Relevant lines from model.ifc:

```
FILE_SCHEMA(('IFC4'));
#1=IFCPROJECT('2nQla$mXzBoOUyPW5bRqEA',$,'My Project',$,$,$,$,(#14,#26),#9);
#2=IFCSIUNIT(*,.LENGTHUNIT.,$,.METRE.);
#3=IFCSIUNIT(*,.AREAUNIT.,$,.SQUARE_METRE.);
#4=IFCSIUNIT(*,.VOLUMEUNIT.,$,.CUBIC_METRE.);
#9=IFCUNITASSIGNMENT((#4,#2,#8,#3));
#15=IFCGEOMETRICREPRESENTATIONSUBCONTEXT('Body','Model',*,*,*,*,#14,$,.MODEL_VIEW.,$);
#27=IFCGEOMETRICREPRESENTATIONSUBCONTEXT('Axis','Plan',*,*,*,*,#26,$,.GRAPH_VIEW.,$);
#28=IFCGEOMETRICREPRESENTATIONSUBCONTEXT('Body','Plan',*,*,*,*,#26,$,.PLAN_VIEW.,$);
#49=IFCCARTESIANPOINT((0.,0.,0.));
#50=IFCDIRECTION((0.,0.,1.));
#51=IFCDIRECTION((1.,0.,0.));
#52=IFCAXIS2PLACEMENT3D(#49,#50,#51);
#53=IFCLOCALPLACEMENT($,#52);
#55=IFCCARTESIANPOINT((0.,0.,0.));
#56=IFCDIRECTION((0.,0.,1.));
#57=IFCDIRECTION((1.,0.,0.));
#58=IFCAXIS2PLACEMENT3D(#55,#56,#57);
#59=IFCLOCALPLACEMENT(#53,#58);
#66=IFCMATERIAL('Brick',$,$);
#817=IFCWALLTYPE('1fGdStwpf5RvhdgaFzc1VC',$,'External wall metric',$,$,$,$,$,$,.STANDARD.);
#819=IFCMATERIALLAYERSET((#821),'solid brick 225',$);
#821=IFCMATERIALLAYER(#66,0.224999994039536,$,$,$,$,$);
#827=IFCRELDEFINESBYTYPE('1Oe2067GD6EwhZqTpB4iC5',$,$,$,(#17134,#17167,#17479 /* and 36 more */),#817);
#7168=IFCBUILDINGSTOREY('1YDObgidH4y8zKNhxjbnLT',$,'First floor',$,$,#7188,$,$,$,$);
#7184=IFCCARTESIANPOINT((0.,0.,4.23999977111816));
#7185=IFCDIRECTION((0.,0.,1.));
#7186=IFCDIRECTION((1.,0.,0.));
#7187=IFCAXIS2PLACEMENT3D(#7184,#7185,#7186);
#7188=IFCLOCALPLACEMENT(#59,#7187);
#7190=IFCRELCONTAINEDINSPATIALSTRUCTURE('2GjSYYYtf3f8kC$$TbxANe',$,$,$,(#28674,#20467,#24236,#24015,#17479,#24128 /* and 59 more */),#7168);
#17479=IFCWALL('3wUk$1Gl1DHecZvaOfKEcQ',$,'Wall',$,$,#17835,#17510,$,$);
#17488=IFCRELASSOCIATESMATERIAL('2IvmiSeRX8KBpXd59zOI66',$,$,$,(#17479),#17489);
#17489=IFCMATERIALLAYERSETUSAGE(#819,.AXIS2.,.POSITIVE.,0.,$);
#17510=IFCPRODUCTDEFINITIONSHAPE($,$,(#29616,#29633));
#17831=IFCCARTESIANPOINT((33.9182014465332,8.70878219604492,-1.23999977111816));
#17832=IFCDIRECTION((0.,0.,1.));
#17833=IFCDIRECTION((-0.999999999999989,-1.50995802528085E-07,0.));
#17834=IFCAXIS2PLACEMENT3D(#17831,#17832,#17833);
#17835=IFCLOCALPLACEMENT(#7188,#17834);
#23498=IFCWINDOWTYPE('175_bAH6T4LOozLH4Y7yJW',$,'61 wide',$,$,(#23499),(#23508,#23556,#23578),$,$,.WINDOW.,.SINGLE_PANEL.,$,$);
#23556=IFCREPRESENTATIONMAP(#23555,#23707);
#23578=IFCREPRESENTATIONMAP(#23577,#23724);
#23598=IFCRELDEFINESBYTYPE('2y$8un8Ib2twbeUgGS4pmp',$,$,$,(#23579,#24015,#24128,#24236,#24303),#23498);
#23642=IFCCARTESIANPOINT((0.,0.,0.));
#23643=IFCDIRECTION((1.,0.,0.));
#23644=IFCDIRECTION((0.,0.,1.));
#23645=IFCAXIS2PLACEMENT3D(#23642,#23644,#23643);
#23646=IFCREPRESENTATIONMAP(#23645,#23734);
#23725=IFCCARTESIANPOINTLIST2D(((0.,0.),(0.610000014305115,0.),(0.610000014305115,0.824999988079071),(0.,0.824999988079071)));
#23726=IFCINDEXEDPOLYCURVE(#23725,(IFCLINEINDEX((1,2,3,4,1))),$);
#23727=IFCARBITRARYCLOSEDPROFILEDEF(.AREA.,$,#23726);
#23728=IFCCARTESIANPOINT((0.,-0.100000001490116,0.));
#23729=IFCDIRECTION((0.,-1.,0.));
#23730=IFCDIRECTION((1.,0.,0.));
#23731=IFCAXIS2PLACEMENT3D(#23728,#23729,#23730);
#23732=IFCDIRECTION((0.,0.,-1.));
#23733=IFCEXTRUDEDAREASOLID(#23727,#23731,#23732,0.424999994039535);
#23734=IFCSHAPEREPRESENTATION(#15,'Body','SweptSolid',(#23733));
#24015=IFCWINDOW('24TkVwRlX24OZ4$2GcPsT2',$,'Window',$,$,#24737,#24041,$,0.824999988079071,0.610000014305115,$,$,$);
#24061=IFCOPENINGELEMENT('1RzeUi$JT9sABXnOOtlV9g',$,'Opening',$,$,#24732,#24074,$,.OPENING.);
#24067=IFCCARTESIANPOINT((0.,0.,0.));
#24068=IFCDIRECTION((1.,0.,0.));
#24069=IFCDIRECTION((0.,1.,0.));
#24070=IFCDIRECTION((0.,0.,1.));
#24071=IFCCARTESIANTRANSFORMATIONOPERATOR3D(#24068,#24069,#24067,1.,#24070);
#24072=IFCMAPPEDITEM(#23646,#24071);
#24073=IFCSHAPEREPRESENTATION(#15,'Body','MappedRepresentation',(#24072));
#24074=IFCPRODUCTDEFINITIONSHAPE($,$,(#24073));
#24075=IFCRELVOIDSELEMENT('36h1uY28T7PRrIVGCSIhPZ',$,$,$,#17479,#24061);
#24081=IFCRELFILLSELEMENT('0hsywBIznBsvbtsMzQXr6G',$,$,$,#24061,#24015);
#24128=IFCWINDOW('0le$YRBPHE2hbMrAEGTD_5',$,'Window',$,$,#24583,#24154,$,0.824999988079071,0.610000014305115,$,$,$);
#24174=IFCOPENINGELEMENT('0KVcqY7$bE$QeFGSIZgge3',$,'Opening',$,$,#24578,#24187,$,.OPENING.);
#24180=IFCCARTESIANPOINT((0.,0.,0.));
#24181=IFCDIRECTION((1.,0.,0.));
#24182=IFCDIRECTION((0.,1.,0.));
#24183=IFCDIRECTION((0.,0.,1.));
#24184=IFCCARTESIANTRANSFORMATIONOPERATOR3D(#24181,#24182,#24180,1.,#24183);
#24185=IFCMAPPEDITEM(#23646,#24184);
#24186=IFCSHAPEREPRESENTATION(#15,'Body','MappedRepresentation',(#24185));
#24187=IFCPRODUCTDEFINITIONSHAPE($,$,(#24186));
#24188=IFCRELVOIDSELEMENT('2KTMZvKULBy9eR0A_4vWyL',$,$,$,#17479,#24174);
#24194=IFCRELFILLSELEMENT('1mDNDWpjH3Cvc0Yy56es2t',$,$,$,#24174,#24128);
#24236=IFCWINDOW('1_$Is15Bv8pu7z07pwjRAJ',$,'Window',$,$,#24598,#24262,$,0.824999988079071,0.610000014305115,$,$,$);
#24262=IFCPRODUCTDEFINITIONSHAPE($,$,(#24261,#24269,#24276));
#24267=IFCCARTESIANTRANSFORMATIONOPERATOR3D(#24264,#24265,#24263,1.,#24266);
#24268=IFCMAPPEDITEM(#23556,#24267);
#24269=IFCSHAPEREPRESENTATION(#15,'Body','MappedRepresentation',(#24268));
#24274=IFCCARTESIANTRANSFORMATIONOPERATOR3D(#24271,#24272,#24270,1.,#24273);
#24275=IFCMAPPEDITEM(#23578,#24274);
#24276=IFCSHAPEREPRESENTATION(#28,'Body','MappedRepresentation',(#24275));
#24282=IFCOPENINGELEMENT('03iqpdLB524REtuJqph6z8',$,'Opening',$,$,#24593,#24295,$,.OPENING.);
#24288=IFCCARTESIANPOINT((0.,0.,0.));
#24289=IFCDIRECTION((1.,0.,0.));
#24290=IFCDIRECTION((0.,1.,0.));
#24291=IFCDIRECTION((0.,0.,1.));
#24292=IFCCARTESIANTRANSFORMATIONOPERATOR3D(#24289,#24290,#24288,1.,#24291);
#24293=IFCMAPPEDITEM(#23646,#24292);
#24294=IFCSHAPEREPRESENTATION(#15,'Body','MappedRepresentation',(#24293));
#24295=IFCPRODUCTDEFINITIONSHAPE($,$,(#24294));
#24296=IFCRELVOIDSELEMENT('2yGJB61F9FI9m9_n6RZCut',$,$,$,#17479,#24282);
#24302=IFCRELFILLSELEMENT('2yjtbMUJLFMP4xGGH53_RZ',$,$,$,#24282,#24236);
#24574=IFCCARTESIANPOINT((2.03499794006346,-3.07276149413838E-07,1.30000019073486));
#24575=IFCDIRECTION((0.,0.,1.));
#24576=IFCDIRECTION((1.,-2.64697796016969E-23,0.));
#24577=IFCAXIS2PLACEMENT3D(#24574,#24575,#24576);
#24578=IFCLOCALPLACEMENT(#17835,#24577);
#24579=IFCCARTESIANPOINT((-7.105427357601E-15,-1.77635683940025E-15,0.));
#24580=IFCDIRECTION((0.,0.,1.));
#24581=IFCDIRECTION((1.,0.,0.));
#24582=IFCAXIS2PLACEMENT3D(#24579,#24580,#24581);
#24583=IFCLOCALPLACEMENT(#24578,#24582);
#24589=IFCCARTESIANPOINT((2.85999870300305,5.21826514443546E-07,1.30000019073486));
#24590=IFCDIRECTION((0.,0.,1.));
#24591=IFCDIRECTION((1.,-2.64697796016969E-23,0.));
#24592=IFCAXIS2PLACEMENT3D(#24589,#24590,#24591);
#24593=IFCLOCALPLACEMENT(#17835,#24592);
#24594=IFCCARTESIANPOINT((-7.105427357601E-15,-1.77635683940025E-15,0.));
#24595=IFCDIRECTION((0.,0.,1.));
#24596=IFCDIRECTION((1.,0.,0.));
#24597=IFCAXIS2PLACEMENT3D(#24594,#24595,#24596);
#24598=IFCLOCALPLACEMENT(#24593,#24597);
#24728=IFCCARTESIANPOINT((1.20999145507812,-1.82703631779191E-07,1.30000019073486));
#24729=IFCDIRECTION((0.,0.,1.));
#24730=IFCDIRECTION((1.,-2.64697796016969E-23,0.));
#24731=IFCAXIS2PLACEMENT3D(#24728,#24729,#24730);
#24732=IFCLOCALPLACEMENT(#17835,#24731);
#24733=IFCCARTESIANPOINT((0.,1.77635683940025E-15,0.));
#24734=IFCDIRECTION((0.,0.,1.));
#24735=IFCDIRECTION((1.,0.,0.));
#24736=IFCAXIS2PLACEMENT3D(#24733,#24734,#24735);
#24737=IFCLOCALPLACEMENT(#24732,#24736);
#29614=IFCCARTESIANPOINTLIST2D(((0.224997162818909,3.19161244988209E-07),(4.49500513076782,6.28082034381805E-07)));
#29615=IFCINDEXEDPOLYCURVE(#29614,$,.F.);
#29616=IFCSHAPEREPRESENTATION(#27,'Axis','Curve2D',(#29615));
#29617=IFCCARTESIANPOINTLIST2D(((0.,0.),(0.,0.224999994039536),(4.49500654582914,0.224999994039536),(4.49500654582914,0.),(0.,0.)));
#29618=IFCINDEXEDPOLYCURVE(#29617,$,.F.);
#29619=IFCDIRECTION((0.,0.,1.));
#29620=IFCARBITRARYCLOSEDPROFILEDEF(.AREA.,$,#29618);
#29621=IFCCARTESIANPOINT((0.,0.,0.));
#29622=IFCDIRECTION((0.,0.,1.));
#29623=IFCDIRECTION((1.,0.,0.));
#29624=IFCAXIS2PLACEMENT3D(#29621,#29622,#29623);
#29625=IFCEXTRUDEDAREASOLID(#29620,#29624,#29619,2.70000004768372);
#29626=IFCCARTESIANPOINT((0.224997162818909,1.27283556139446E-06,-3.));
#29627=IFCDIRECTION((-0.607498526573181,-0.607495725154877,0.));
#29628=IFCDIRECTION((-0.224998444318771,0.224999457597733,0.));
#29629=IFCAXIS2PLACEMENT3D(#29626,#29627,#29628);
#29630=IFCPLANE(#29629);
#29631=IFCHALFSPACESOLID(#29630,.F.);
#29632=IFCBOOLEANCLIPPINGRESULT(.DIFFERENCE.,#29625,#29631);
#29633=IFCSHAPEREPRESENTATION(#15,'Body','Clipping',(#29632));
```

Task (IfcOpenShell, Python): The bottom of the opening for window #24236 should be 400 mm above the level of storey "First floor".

```python
import numpy as np
import ifcopenshell
import ifcopenshell.api.geometry
import ifcopenshell.geom
import ifcopenshell.util.element
import ifcopenshell.util.placement
import ifcopenshell.util.shape
import ifcopenshell.util.unit

model = ifcopenshell.open("model.ifc")
unit_scale = ifcopenshell.util.unit.calculate_unit_scale(model)

window = model.by_id(24236)
opening = window.FillsVoids[0].RelatingOpeningElement
storey = ifcopenshell.util.element.get_container(window, ifc_class="IfcBuildingStorey")
level = ifcopenshell.util.placement.get_local_placement(storey.ObjectPlacement)[2, 3]

# The opening's origin need not be at the sill, so measure its lowest point.
shape = ifcopenshell.geom.create_shape(ifcopenshell.geom.settings(), opening)
bottom = ifcopenshell.util.shape.get_shape_bottom_elevation(shape, shape.geometry) / unit_scale
dz = level + 0.4 / unit_scale - bottom

shift = np.array([0.0, 0.0, dz])
# The window is placed relative to its opening, so it follows when the opening moves.
matrix = ifcopenshell.util.placement.get_local_placement(opening.ObjectPlacement)
matrix[:3, 3] += shift
ifcopenshell.api.geometry.edit_object_placement(
    model, product=opening, matrix=matrix, is_si=False, should_transform_children=True
)

print(f"moved by {dz * unit_scale:+.3f} m")

model.write("model_v2.ifc")
```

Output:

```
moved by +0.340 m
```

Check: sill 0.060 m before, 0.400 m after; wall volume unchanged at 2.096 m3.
